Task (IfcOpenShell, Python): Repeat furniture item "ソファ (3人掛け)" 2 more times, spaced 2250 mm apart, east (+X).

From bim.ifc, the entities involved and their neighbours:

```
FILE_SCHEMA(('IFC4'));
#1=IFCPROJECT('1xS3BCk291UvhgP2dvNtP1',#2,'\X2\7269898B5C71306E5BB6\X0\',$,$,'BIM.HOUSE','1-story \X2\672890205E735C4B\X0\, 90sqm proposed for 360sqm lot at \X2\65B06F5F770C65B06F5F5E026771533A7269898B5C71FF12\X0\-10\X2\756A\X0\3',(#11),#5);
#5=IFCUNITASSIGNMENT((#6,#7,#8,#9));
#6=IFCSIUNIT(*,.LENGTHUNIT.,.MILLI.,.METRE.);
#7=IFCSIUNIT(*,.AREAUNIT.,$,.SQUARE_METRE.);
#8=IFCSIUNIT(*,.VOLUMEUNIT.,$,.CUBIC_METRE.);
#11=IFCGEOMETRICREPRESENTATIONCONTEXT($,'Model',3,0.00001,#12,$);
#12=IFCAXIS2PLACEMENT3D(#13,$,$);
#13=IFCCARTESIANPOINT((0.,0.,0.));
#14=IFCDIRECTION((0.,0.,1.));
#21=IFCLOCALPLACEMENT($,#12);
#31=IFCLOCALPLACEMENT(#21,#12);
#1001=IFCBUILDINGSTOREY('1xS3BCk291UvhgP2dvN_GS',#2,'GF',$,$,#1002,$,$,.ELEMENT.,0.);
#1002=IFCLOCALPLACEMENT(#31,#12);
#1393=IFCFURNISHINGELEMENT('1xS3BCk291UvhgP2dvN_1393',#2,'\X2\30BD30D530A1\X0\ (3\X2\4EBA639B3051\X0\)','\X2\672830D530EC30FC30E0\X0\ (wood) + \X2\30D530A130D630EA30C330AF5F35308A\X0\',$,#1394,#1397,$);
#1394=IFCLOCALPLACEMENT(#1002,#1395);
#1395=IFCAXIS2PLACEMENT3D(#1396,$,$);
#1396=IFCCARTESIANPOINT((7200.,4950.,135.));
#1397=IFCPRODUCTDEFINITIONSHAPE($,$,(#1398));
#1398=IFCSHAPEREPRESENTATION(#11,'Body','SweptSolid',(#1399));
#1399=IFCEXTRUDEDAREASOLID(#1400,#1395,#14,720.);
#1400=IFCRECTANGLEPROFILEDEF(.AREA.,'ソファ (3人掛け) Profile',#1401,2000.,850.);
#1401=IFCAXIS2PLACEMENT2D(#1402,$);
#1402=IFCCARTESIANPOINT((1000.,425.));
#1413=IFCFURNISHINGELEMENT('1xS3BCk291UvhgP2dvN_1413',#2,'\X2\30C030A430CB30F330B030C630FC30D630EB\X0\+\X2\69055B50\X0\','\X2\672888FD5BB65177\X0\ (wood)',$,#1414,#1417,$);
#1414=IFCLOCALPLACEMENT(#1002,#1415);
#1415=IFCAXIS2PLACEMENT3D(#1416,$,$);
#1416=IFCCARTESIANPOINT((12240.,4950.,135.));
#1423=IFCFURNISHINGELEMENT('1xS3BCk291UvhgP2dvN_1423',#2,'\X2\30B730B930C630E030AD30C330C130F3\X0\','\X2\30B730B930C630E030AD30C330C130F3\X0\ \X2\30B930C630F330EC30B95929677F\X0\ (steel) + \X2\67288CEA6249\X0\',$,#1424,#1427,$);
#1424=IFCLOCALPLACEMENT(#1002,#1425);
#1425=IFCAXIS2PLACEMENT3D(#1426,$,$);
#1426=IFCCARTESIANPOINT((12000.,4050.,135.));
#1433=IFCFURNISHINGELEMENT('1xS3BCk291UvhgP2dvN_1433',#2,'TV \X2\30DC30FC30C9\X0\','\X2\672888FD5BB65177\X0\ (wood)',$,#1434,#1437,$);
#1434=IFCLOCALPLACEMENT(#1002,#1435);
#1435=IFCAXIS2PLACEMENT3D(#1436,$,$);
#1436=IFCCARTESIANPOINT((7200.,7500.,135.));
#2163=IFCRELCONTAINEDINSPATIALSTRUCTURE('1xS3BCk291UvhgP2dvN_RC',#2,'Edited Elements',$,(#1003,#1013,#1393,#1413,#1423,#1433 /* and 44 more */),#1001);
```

```python
import numpy as np
import ifcopenshell
import ifcopenshell.api.geometry
import ifcopenshell.api.root
import ifcopenshell.util.element
import ifcopenshell.util.placement

model = ifcopenshell.open("bim.ifc")


def reuse_history(source, copy):
    """copy_class also copies each property set's owner history, people and application; keep the originals."""
    for rel in copy.IsDefinedBy:
        if rel.is_a("IfcRelDefinesByProperties") and (history := rel.RelatingPropertyDefinition.OwnerHistory):
            rel.RelatingPropertyDefinition.OwnerHistory = source.OwnerHistory
            ifcopenshell.util.element.remove_deep2(model, history)


source = model.by_guid("1xS3BCk291UvhgP2dvN_1393")
base = ifcopenshell.util.placement.get_local_placement(source.ObjectPlacement)
step = np.array([1.0, 0.0, 0.0]) * 2250.0

for i in range(1, 3):
    copy = ifcopenshell.api.root.copy_class(model, product=source)
    copy.Representation = ifcopenshell.util.element.copy_deep(
        model, source.Representation, exclude=["IfcGeometricRepresentationContext", "IfcRepresentationMap"]
    )
    reuse_history(source, copy)
    matrix = base.copy()
    matrix[:3, 3] += i * step
    print("added at", matrix[:3, 3].round(3) + 0.0)
    ifcopenshell.api.geometry.edit_object_placement(model, product=copy, matrix=matrix, is_si=False)

model.write("bim_updated.ifc")
```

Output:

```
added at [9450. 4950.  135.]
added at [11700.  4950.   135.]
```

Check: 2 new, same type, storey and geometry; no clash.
